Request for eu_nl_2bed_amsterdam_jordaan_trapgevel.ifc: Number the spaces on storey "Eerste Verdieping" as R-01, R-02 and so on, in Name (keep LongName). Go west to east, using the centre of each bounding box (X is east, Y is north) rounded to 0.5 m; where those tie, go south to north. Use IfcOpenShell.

First a look at what the model holds.

```python
import ifcopenshell
import ifcopenshell.util.element
import ifcopenshell.util.placement

model = ifcopenshell.open("eu_nl_2bed_amsterdam_jordaan_trapgevel.ifc")
print(model.schema)
storey = next(s for s in model.by_type("IfcBuildingStorey") if s.Name == "Eerste Verdieping")
spaces = [e for e in ifcopenshell.util.element.get_decomposition(storey) if e.is_a("IfcSpace")]
for e in sorted(spaces, key=lambda e: e.id()):
    origin = ifcopenshell.util.placement.get_local_placement(e.ObjectPlacement)[:3, 3]
    print(e.id(), e.Name, e.LongName, origin.round(2) + 0.0, sep=" | ")
```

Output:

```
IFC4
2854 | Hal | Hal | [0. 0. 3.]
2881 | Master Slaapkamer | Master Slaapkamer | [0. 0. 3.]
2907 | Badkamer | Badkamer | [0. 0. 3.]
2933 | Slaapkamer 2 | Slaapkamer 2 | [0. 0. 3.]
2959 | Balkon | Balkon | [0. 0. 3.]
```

```python
import ifcopenshell
import ifcopenshell.geom
import ifcopenshell.util.element
import ifcopenshell.util.shape

model = ifcopenshell.open("eu_nl_2bed_amsterdam_jordaan_trapgevel.ifc")
settings = ifcopenshell.geom.settings()
settings.set("use-world-coords", True)


def centre(element):
    shape = ifcopenshell.geom.create_shape(settings, element)
    return ifcopenshell.util.shape.get_bbox_centroid(shape.geometry)


storey = next(s for s in model.by_type("IfcBuildingStorey") if s.Name == "Eerste Verdieping")
spaces = [e for e in ifcopenshell.util.element.get_decomposition(storey) if e.is_a("IfcSpace")]

# Insertion points can sit at a corner or the storey origin, so sort by the geometry (in metres).
centres = {e: centre(e) for e in spaces}
spaces.sort(key=lambda e: (round(centres[e][0] / 0.5), centres[e][1]))

for i, e in enumerate(spaces, start=1):
    number = f"R-{i:02d}"
    e.Name = number
    print(e.id(), number)

model.write("eu_nl_2bed_amsterdam_jordaan_trapgevel_rev.ifc")
```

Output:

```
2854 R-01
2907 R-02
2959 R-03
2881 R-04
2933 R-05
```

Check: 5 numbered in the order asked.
